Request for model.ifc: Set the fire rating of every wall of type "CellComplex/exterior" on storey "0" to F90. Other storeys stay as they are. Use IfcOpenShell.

First a look at what the model holds.

```python
import ifcopenshell
import ifcopenshell.util.element

model = ifcopenshell.open("model.ifc")
print(model.schema)
storey = next(s for s in model.by_type("IfcBuildingStorey") if s.Name == "0")
walls = [e for e in ifcopenshell.util.element.get_decomposition(storey) if e.is_a("IfcWall")]
seen = {}
for e in walls:
    element_type = ifcopenshell.util.element.get_type(e)
    key = (element_type.Name if element_type != e and element_type else None, ifcopenshell.util.element.get_pset(e, "Pset_WallCommon", "FireRating"))
    seen[key] = seen.get(key, 0) + 1
for (name, value), count in sorted(seen.items(), key=str):
    print(count, "x", name, "|", value)
```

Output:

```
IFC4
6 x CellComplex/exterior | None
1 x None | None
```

```python
import ifcopenshell
import ifcopenshell.api.pset
import ifcopenshell.util.element

model = ifcopenshell.open("model.ifc")

storey = next(s for s in model.by_type("IfcBuildingStorey") if s.Name == "0")
walls = [e for e in ifcopenshell.util.element.get_decomposition(storey) if e.is_a("IfcWall")]

count = 0
for e in walls:
    element_type = ifcopenshell.util.element.get_type(e)
    if element_type in (None, e) or element_type.Name != "CellComplex/exterior":
        continue
    # add_pset returns the element's existing set when there is one.
    pset = ifcopenshell.api.pset.add_pset(model, product=e, name="Pset_WallCommon")
    ifcopenshell.api.pset.edit_pset(model, pset=pset, properties={"FireRating": "F90"})
    count += 1

print(count, "walls updated")

model.write("model_rev.ifc")
```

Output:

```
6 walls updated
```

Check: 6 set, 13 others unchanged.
